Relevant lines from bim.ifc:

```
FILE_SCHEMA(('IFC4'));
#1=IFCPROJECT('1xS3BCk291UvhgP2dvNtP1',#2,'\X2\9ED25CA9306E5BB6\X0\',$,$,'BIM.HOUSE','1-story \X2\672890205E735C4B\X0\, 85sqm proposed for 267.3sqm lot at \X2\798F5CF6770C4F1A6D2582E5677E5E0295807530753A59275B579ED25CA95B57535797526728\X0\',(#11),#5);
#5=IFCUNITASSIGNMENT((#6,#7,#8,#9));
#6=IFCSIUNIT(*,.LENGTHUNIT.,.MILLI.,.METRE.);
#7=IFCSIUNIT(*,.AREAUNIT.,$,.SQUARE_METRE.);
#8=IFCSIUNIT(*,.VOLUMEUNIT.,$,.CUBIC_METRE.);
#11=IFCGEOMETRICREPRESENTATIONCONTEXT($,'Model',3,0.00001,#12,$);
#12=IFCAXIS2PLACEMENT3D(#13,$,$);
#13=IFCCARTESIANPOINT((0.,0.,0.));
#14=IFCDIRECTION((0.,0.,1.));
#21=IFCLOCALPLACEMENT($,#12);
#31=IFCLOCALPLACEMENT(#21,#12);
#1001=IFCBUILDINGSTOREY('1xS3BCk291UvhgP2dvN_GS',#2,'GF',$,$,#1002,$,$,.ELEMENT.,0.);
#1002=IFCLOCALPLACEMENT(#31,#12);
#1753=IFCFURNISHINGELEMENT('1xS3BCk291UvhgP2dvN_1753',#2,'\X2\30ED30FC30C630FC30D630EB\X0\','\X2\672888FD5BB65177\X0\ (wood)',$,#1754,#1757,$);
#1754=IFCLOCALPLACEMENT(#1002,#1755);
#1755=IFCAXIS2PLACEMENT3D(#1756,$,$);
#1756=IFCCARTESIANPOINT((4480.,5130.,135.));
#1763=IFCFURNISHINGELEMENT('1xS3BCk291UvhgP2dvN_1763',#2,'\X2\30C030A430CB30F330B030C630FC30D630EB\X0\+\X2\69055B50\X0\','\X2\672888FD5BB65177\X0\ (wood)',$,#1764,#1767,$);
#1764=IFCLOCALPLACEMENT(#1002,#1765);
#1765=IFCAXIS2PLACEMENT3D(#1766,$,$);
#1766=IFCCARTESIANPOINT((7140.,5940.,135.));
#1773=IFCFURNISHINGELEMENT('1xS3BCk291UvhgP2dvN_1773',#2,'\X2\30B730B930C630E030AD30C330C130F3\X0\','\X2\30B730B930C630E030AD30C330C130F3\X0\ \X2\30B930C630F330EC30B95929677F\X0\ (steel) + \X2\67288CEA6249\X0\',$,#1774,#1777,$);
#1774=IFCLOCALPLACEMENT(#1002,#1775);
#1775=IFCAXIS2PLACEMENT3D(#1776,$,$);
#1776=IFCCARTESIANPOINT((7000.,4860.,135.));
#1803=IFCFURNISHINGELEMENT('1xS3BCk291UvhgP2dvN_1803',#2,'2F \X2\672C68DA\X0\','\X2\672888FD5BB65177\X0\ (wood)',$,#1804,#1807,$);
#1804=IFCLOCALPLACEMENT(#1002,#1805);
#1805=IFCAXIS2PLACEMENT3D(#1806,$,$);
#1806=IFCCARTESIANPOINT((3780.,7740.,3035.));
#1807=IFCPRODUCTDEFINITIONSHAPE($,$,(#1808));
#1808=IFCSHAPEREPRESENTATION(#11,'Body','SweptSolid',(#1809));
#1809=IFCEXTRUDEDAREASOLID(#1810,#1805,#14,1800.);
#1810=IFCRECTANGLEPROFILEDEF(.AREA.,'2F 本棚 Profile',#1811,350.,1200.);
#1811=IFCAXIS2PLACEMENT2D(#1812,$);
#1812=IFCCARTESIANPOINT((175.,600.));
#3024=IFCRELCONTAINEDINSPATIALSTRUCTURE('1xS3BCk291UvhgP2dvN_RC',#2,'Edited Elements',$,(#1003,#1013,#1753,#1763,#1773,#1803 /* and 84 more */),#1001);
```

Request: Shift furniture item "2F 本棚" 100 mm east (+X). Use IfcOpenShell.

```python
import ifcopenshell
import ifcopenshell.api.geometry
import ifcopenshell.util.placement

model = ifcopenshell.open("bim.ifc")

item = model.by_id(1803)
matrix = ifcopenshell.util.placement.get_local_placement(item.ObjectPlacement)
matrix[0, 3] += 100.0
ifcopenshell.api.geometry.edit_object_placement(model, product=item, matrix=matrix, is_si=False)

print(ifcopenshell.util.placement.get_local_placement(item.ObjectPlacement).round(3) + 0.0)

model.write("bim_v2.ifc")
```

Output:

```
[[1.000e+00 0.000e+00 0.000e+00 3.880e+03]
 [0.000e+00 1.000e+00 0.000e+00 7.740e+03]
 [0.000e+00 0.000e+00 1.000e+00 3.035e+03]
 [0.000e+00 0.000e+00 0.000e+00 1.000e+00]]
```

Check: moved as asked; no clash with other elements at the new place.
